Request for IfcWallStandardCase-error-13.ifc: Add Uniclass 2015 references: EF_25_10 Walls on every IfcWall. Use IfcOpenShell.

First a look at what the model holds.

```python
import ifcopenshell

model = ifcopenshell.open("IfcWallStandardCase-error-13.ifc")
print(model.schema)
print("classifications:", [c.Name for c in model.by_type("IfcClassification")])
for ifc_class in ("IfcDoor", "IfcRoof", "IfcStair", "IfcWall", "IfcWindow"):
    print(ifc_class, len(model.by_type(ifc_class)))
```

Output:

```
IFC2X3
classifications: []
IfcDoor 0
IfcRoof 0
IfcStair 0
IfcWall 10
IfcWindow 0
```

```python
import ifcopenshell
import ifcopenshell.api.classification

model = ifcopenshell.open("IfcWallStandardCase-error-13.ifc")

# IFC2X3 requires Source and Edition and has no link from the project to the system.
system = model.create_entity("IfcClassification", Source="NBS", Edition="2015", Name="Uniclass 2015")

codes = {
    "IfcWall": ("EF_25_10", "Walls"),
}
for ifc_class, (code, name) in codes.items():
    products = model.by_type(ifc_class)
    ifcopenshell.api.classification.add_reference(
        model, products=products, classification=system, identification=code, name=name
    )
    print(code, len(products))

model.write("IfcWallStandardCase-error-13_updated.ifc")
```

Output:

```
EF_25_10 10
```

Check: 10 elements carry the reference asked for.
